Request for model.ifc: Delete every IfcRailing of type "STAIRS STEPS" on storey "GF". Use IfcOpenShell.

First a look at what the model holds.

```python
import ifcopenshell
import ifcopenshell.util.element

model = ifcopenshell.open("model.ifc")
print(model.schema)
storey = next(s for s in model.by_type("IfcBuildingStorey") if s.Name == "GF")
railings = [e for e in ifcopenshell.util.element.get_decomposition(storey) if e.is_a("IfcRailing")]
seen = {}
for e in railings:
    element_type = ifcopenshell.util.element.get_type(e)
    name = element_type.Name if element_type not in (None, e) else None
    seen[name] = seen.get(name, 0) + 1
for name, count in sorted(seen.items(), key=str):
    print(count, "x", name)
```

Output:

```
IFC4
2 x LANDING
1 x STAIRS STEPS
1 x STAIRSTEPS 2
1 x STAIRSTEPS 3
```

```python
import ifcopenshell
import ifcopenshell.api.root
import ifcopenshell.util.element

model = ifcopenshell.open("model.ifc")

storey = next(s for s in model.by_type("IfcBuildingStorey") if s.Name == "GF")
railings = [e for e in ifcopenshell.util.element.get_decomposition(storey) if e.is_a("IfcRailing")]
targets = [e for e in railings if (t := ifcopenshell.util.element.get_type(e)) not in (None, e) and t.Name == "STAIRS STEPS"]

for e in targets:
    ifcopenshell.api.root.remove_product(model, product=e)
print(len(targets), "removed")

model.write("model_edited.ifc")
```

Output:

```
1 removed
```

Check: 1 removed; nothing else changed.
